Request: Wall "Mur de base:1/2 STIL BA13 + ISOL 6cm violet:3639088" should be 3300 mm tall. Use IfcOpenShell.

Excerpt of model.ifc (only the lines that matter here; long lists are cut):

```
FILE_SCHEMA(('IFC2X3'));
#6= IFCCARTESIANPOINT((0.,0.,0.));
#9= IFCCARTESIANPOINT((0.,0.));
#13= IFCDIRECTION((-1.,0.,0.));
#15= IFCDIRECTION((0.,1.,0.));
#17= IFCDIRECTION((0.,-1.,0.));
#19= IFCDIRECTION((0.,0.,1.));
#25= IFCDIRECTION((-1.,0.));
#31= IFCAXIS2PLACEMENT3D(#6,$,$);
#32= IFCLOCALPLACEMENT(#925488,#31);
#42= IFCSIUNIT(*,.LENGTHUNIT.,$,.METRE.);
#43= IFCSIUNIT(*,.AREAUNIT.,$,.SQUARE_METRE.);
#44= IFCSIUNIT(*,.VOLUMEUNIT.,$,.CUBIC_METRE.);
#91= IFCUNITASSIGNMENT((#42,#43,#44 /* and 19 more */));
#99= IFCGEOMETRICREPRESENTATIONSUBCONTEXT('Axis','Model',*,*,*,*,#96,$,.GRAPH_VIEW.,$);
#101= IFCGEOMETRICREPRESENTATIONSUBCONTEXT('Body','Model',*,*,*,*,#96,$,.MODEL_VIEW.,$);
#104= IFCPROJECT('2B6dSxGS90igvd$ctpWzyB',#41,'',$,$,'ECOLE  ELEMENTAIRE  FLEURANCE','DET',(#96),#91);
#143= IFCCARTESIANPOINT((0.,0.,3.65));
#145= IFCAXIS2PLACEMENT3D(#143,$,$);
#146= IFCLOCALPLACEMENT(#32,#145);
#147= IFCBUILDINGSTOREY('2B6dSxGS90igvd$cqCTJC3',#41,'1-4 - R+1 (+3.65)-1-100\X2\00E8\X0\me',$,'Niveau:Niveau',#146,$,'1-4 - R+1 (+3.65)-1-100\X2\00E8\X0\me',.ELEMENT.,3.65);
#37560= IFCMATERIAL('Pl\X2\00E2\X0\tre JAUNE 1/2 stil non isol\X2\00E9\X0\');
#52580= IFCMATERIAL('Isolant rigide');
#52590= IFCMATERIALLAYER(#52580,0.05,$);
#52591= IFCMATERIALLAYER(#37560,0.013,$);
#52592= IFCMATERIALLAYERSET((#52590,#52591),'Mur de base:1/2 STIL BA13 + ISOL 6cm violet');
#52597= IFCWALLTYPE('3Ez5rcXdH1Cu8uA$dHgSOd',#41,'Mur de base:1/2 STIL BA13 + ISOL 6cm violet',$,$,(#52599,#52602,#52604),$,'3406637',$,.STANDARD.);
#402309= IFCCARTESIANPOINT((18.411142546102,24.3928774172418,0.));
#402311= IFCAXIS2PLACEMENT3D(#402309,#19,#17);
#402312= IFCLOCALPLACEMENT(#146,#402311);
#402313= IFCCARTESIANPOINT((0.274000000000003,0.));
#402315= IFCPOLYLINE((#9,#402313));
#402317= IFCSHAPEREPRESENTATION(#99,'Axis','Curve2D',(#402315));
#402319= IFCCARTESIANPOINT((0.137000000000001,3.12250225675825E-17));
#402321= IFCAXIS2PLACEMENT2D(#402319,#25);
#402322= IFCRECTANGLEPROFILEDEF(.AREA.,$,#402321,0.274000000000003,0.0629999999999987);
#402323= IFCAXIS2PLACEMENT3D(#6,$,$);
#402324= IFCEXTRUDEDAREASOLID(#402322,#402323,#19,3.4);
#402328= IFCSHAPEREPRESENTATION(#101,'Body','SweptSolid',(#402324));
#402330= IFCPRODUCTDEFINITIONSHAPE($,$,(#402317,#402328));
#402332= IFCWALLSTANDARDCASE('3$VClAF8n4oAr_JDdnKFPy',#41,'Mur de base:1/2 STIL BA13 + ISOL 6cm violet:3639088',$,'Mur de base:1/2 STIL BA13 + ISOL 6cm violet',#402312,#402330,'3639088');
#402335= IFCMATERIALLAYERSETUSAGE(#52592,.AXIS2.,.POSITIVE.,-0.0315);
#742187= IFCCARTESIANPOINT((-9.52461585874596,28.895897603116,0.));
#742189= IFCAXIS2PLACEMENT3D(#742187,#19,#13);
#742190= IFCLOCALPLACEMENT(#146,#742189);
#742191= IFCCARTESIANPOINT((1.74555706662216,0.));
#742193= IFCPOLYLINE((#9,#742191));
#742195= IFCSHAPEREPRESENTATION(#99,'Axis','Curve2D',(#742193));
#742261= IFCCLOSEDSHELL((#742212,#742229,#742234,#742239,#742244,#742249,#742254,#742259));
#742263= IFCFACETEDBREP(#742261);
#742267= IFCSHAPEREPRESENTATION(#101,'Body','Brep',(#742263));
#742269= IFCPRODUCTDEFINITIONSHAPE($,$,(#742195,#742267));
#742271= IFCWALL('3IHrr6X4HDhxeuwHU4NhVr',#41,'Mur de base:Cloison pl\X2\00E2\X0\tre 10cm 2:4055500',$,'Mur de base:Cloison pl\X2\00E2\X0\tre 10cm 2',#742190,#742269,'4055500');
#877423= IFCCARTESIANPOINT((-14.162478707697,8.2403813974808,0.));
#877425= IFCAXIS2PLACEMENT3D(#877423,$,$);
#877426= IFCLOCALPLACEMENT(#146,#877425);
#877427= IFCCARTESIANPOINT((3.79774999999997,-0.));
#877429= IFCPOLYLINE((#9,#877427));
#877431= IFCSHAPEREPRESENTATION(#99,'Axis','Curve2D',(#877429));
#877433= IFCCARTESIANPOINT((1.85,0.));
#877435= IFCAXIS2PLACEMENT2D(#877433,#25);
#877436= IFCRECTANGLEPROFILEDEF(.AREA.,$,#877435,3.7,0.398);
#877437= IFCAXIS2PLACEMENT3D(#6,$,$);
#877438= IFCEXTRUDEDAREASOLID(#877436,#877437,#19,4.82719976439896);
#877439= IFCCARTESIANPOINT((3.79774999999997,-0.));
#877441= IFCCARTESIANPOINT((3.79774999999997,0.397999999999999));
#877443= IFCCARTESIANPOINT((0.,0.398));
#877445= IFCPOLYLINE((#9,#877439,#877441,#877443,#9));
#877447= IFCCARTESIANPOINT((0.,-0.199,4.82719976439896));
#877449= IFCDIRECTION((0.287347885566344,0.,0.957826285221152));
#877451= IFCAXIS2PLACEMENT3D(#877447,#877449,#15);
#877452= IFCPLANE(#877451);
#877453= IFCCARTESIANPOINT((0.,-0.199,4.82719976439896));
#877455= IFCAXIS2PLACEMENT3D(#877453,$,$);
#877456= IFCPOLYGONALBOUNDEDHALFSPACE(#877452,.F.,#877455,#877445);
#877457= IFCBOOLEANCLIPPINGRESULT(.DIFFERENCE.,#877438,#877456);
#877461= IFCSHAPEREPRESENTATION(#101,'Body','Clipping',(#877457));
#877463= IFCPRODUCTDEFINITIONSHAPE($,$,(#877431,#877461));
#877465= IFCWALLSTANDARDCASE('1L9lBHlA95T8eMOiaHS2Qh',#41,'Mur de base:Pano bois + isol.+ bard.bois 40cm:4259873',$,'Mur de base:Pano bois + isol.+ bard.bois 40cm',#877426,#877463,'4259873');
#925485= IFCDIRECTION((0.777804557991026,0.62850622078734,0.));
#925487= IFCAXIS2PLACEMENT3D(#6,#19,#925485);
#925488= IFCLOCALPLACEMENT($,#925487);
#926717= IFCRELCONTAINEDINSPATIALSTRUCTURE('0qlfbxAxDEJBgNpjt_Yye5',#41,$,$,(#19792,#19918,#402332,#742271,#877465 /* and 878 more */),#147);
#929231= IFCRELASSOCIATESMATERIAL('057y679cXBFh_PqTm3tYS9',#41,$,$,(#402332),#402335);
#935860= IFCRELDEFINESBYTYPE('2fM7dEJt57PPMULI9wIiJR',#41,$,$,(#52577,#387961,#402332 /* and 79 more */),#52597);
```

```python
import ifcopenshell
import ifcopenshell.geom
import ifcopenshell.util.representation
import ifcopenshell.util.shape
import ifcopenshell.util.unit

model = ifcopenshell.open("model.ifc")
unit_scale = ifcopenshell.util.unit.calculate_unit_scale(model)
settings = ifcopenshell.geom.settings()


def volume(element):
    """Net volume in cubic metres, openings subtracted."""
    shape = ifcopenshell.geom.create_shape(settings, element)
    return ifcopenshell.util.shape.get_volume(shape.geometry)


wall = model.by_guid("3$VClAF8n4oAr_JDdnKFPy")
before = volume(wall)

body = ifcopenshell.util.representation.get_representation(wall, "Model", "Body")
solid = body.Items[0]
old_height = solid.Depth
solid.Depth = 3.3 / unit_scale
after = volume(wall)

print(f"height {old_height:g} -> {solid.Depth:g}, volume {before:.3f} -> {after:.3f} m3")

model.write("model_updated.ifc")
```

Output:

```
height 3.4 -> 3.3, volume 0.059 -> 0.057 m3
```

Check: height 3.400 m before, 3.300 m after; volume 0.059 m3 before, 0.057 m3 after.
